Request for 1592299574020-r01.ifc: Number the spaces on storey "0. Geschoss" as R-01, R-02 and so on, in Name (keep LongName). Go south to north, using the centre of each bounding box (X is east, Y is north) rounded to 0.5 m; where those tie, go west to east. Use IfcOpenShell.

First a look at what the model holds.

```python
import ifcopenshell
import ifcopenshell.util.element
import ifcopenshell.util.placement

model = ifcopenshell.open("1592299574020-r01.ifc")
print(model.schema)
storey = next(s for s in model.by_type("IfcBuildingStorey") if s.Name == "0. Geschoss")
spaces = [e for e in ifcopenshell.util.element.get_decomposition(storey) if e.is_a("IfcSpace")]
for e in sorted(spaces, key=lambda e: e.id()):
    origin = ifcopenshell.util.placement.get_local_placement(e.ObjectPlacement)[:3, 3]
    print(e.id(), e.Name, e.LongName, origin.round(2) + 0.0, sep=" | ")
```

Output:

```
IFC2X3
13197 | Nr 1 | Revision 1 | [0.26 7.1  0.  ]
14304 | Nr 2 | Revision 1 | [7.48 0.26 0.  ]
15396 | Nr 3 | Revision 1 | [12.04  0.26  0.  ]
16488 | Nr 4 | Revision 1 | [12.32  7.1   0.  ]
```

```python
import ifcopenshell
import ifcopenshell.geom
import ifcopenshell.util.element
import ifcopenshell.util.shape

model = ifcopenshell.open("1592299574020-r01.ifc")
settings = ifcopenshell.geom.settings()
settings.set("use-world-coords", True)


def centre(element):
    shape = ifcopenshell.geom.create_shape(settings, element)
    return ifcopenshell.util.shape.get_bbox_centroid(shape.geometry)


storey = next(s for s in model.by_type("IfcBuildingStorey") if s.Name == "0. Geschoss")
spaces = [e for e in ifcopenshell.util.element.get_decomposition(storey) if e.is_a("IfcSpace")]

# Insertion points can sit at a corner or the storey origin, so sort by the geometry (in metres).
centres = {e: centre(e) for e in spaces}
spaces.sort(key=lambda e: (round(centres[e][1] / 0.5), centres[e][0]))

for i, e in enumerate(spaces, start=1):
    number = f"R-{i:02d}"
    e.Name = number
    print(e.id(), number)

model.write("1592299574020-r01_updated.ifc")
```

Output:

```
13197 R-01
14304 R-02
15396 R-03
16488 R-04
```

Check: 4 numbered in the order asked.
